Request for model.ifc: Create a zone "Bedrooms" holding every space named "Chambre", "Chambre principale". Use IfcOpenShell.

First a look at what the model holds.

```python
import ifcopenshell

model = ifcopenshell.open("model.ifc")
print(model.schema)
seen = {}
for space in model.by_type("IfcSpace"):
    seen[space.LongName] = seen.get(space.LongName, 0) + 1
for name, count in sorted(seen.items(), key=str):
    print(count, "x", name)
print("zones:", [z.Name for z in model.by_type("IfcZone")][:20])
```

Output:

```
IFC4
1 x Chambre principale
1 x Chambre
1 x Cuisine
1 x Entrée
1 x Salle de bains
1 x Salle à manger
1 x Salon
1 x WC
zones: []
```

```python
import ifcopenshell
import ifcopenshell.api.group
import ifcopenshell.api.root

model = ifcopenshell.open("model.ifc")

names = {"Chambre", "Chambre principale"}
spaces = [s for s in model.by_type("IfcSpace") if s.LongName in names]

zone = ifcopenshell.api.root.create_entity(model, ifc_class="IfcZone", name="Bedrooms")
ifcopenshell.api.group.assign_group(model, products=spaces, group=zone)
print(len(spaces), "spaces in", zone.Name)

model.write("model_rev.ifc")
```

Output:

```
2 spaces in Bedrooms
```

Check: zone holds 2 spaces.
